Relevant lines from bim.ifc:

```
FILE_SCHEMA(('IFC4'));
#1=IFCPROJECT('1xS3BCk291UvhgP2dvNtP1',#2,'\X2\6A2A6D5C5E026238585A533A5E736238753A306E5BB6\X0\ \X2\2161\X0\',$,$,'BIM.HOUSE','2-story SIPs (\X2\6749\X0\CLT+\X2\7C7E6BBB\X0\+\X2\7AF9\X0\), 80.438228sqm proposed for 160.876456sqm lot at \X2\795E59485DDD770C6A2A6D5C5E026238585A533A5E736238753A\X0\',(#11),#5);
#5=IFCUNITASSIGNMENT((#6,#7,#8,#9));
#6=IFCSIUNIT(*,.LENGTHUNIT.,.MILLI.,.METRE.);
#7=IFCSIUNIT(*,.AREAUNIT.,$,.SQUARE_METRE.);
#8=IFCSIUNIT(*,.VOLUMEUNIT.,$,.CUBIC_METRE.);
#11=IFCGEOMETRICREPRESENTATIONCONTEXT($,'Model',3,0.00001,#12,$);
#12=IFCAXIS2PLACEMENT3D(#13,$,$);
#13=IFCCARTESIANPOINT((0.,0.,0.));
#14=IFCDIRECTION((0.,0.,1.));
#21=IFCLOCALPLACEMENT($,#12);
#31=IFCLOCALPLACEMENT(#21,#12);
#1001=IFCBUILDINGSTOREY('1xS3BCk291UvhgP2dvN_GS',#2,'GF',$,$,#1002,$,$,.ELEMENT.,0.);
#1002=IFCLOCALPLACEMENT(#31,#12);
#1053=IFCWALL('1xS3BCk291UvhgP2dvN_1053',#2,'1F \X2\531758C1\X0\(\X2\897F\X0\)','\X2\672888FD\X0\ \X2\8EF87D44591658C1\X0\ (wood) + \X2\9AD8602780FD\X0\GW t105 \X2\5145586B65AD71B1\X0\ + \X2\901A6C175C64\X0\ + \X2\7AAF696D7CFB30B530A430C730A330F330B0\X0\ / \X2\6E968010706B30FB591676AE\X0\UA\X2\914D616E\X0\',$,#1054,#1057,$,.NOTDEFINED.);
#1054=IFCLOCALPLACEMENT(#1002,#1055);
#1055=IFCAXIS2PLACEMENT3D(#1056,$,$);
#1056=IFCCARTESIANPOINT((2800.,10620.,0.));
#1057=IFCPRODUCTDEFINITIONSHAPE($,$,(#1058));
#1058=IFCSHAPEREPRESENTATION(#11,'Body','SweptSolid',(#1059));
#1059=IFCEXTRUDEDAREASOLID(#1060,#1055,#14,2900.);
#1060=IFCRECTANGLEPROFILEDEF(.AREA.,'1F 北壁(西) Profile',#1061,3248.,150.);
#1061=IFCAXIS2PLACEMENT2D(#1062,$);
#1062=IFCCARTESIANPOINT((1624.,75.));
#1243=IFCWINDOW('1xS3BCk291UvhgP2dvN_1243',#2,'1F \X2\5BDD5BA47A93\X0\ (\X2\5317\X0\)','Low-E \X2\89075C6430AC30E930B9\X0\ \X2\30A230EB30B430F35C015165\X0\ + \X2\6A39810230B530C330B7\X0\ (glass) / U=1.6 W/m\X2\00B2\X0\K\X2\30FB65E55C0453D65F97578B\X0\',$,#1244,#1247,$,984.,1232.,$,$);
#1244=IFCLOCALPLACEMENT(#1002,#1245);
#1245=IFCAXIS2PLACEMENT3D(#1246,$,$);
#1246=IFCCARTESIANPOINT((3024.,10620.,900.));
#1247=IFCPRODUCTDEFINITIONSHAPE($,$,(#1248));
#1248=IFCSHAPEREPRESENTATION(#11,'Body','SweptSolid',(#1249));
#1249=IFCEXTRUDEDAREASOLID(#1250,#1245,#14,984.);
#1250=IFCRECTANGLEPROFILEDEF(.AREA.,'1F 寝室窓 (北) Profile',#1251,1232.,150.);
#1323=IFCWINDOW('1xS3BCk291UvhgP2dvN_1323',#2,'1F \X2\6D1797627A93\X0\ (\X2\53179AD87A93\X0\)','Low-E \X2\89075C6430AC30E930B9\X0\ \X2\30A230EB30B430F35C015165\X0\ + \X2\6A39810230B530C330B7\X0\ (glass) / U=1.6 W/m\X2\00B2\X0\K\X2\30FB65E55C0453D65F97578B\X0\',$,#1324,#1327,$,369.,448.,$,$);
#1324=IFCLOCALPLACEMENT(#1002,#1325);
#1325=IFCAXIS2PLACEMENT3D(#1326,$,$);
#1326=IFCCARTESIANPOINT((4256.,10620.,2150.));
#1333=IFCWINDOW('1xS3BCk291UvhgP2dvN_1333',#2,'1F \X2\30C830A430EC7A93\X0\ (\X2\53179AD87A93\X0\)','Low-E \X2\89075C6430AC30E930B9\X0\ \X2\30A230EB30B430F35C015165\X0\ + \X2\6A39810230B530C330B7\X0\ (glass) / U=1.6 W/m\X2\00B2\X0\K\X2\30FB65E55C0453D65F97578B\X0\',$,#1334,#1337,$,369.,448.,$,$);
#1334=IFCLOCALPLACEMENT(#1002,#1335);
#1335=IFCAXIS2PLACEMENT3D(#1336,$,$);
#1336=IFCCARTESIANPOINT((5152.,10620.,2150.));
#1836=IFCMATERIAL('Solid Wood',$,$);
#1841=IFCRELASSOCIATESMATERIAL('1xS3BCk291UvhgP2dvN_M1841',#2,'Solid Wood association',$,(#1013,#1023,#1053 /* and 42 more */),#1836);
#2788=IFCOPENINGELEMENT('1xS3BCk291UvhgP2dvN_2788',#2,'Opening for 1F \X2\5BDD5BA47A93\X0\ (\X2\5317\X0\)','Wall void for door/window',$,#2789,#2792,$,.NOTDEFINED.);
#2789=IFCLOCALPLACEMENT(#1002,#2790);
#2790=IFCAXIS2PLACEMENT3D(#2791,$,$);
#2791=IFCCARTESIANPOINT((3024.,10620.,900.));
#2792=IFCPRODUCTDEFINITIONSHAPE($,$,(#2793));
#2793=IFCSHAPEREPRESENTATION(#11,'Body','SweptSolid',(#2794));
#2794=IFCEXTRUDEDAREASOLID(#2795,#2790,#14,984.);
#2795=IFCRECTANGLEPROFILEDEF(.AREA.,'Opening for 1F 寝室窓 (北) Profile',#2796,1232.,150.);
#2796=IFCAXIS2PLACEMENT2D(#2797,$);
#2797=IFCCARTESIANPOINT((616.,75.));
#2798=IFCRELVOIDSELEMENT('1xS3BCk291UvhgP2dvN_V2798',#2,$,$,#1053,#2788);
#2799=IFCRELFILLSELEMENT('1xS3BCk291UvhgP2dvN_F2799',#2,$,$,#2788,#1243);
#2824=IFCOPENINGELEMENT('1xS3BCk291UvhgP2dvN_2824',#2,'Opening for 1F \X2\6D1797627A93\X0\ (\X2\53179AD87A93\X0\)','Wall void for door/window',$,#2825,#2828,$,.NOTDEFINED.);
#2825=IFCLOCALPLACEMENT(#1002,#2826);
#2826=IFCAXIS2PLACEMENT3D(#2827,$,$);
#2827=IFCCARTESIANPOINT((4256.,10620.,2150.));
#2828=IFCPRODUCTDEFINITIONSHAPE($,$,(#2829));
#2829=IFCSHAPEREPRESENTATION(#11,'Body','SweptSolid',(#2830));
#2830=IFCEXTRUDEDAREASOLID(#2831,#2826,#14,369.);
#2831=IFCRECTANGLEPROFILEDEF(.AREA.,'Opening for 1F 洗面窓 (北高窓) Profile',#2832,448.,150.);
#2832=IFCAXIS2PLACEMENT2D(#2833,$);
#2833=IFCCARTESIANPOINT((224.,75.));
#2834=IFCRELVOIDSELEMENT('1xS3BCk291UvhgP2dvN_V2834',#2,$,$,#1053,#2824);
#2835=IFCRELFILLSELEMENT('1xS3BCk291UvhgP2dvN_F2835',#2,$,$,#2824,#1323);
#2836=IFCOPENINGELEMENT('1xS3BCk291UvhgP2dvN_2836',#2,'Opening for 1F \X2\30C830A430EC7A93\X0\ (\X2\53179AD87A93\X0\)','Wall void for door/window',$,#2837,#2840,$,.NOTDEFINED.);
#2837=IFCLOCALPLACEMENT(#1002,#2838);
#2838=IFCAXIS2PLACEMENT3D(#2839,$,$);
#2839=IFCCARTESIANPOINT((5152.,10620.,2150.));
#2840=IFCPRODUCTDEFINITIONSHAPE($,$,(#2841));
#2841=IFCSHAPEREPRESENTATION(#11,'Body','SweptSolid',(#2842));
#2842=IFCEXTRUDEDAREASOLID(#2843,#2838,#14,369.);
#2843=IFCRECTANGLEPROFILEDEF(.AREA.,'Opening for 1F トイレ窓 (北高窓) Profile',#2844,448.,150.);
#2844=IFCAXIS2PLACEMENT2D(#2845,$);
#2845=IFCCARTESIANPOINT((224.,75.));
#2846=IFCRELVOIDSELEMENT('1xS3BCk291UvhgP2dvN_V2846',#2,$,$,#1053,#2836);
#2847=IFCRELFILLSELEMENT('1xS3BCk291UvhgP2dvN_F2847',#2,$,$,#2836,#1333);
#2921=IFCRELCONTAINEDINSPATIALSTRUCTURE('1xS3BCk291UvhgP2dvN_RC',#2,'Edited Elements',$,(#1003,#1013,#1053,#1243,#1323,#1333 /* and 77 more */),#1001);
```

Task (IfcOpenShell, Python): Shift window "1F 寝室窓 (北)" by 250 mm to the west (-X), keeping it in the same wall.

```python
import ifcopenshell
import ifcopenshell.api.geometry
import ifcopenshell.util.placement
import ifcopenshell.util.unit

model = ifcopenshell.open("bim.ifc")
unit_scale = ifcopenshell.util.unit.calculate_unit_scale(model)

window = model.by_id(1243)
opening = window.FillsVoids[0].RelatingOpeningElement
wall = opening.VoidsElements[0].RelatingBuildingElement

wall_matrix = ifcopenshell.util.placement.get_local_placement(wall.ObjectPlacement)
shift = wall_matrix[:3, 0] * -0.25 / unit_scale
before = ifcopenshell.util.placement.get_local_placement(window.ObjectPlacement)[:3, 3].copy()

# The window is not placed relative to its opening, so move both.
for product in (opening, window):
    matrix = ifcopenshell.util.placement.get_local_placement(product.ObjectPlacement)
    matrix[:3, 3] += shift
    ifcopenshell.api.geometry.edit_object_placement(model, product=product, matrix=matrix, is_si=False)

after = ifcopenshell.util.placement.get_local_placement(window.ObjectPlacement)[:3, 3]
print("window moved by", (after - before).round(3) + 0.0)

model.write("bim-out.ifc")
```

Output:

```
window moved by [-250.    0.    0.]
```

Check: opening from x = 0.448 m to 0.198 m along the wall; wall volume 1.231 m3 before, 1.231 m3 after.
